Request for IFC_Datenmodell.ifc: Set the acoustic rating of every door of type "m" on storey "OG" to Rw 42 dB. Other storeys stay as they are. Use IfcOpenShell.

First a look at what the model holds.

```python
import ifcopenshell
import ifcopenshell.util.element

model = ifcopenshell.open("IFC_Datenmodell.ifc")
print(model.schema)
storey = next(s for s in model.by_type("IfcBuildingStorey") if s.Name == "OG")
doors = [e for e in ifcopenshell.util.element.get_decomposition(storey) if e.is_a("IfcDoor")]
seen = {}
for e in doors:
    element_type = ifcopenshell.util.element.get_type(e)
    key = (element_type.Name if element_type != e and element_type else None, ifcopenshell.util.element.get_pset(e, "Pset_DoorCommon", "AcousticRating"))
    seen[key] = seen.get(key, 0) + 1
for (name, value), count in sorted(seen.items(), key=str):
    print(count, "x", name, "|", value)
```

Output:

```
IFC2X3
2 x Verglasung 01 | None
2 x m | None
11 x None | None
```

```python
import ifcopenshell
import ifcopenshell.api.pset
import ifcopenshell.util.element

model = ifcopenshell.open("IFC_Datenmodell.ifc")

storey = next(s for s in model.by_type("IfcBuildingStorey") if s.Name == "OG")
doors = [e for e in ifcopenshell.util.element.get_decomposition(storey) if e.is_a("IfcDoor")]

count = 0
for e in doors:
    element_type = ifcopenshell.util.element.get_type(e)
    if element_type in (None, e) or element_type.Name != "m":
        continue
    # add_pset returns the element's existing set when there is one.
    pset = ifcopenshell.api.pset.add_pset(model, product=e, name="Pset_DoorCommon")
    ifcopenshell.api.pset.edit_pset(model, pset=pset, properties={"AcousticRating": "Rw 42 dB"})
    count += 1

print(count, "doors updated")

model.write("IFC_Datenmodell_updated.ifc")
```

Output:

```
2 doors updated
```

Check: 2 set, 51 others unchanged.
